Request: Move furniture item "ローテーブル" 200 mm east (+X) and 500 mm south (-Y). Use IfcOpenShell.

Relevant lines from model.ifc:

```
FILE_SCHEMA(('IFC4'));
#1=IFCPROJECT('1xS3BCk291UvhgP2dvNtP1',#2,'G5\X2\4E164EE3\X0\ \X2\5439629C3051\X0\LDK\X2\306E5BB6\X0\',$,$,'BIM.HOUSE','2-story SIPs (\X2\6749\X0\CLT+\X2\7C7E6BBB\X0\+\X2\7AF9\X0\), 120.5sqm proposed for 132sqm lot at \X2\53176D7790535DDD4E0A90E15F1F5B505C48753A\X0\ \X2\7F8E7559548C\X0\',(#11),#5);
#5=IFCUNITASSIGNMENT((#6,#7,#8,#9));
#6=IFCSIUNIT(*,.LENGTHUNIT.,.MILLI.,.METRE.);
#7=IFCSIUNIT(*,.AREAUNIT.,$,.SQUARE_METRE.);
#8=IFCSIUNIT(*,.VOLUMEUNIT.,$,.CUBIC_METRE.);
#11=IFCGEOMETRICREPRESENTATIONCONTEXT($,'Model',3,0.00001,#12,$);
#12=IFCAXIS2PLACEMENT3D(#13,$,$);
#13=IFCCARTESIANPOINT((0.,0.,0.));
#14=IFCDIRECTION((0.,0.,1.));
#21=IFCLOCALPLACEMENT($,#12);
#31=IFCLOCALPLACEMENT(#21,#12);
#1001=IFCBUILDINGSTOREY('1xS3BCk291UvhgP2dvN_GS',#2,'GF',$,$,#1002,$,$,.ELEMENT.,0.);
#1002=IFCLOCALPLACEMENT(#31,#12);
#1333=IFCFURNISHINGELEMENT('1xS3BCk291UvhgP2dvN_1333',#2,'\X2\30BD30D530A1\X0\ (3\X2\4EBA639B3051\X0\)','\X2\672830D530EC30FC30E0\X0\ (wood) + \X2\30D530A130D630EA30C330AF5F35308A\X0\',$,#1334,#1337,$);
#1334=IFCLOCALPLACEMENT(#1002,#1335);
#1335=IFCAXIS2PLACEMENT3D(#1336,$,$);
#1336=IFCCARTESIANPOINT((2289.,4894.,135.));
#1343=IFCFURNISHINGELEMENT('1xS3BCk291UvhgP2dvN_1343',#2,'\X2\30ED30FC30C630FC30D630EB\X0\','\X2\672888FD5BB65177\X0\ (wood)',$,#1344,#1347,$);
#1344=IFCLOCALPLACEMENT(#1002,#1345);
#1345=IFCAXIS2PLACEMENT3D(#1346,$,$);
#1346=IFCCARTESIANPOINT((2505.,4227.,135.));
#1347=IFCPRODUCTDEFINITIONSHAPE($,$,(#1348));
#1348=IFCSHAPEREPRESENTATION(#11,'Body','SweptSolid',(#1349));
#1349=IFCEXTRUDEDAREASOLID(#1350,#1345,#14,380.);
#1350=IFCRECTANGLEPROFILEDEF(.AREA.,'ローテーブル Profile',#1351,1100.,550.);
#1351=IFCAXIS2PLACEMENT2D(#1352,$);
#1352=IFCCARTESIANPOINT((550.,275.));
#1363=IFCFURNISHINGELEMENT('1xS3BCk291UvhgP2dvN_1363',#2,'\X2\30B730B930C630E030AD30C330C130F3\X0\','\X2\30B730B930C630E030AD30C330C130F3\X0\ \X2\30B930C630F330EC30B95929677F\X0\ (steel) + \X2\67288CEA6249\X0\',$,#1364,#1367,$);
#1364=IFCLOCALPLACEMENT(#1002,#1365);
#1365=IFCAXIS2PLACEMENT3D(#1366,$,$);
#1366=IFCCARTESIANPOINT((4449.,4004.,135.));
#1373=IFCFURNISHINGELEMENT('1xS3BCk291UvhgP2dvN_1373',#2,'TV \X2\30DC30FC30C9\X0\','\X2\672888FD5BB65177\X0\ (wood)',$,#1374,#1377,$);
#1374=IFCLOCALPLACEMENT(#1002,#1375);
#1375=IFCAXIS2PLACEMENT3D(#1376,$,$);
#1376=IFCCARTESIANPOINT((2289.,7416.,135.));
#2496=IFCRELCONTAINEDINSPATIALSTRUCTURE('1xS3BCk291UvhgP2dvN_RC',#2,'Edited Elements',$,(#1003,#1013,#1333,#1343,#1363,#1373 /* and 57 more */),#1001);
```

```python
import ifcopenshell
import ifcopenshell.api.geometry
import ifcopenshell.util.placement
import ifcopenshell.util.unit

model = ifcopenshell.open("model.ifc")
unit_scale = ifcopenshell.util.unit.calculate_unit_scale(model)

item = model.by_guid("1xS3BCk291UvhgP2dvN_1343")
matrix = ifcopenshell.util.placement.get_local_placement(item.ObjectPlacement)
matrix[0, 3] += 0.2 / unit_scale
matrix[1, 3] -= 0.5 / unit_scale
ifcopenshell.api.geometry.edit_object_placement(model, product=item, matrix=matrix, is_si=False)

print(ifcopenshell.util.placement.get_local_placement(item.ObjectPlacement).round(3) + 0.0)

model.write("model_rev.ifc")
```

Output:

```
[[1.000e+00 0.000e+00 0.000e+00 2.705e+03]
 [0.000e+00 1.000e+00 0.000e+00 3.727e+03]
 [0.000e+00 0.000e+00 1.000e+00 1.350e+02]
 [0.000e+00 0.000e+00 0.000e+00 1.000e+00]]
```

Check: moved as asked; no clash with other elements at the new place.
